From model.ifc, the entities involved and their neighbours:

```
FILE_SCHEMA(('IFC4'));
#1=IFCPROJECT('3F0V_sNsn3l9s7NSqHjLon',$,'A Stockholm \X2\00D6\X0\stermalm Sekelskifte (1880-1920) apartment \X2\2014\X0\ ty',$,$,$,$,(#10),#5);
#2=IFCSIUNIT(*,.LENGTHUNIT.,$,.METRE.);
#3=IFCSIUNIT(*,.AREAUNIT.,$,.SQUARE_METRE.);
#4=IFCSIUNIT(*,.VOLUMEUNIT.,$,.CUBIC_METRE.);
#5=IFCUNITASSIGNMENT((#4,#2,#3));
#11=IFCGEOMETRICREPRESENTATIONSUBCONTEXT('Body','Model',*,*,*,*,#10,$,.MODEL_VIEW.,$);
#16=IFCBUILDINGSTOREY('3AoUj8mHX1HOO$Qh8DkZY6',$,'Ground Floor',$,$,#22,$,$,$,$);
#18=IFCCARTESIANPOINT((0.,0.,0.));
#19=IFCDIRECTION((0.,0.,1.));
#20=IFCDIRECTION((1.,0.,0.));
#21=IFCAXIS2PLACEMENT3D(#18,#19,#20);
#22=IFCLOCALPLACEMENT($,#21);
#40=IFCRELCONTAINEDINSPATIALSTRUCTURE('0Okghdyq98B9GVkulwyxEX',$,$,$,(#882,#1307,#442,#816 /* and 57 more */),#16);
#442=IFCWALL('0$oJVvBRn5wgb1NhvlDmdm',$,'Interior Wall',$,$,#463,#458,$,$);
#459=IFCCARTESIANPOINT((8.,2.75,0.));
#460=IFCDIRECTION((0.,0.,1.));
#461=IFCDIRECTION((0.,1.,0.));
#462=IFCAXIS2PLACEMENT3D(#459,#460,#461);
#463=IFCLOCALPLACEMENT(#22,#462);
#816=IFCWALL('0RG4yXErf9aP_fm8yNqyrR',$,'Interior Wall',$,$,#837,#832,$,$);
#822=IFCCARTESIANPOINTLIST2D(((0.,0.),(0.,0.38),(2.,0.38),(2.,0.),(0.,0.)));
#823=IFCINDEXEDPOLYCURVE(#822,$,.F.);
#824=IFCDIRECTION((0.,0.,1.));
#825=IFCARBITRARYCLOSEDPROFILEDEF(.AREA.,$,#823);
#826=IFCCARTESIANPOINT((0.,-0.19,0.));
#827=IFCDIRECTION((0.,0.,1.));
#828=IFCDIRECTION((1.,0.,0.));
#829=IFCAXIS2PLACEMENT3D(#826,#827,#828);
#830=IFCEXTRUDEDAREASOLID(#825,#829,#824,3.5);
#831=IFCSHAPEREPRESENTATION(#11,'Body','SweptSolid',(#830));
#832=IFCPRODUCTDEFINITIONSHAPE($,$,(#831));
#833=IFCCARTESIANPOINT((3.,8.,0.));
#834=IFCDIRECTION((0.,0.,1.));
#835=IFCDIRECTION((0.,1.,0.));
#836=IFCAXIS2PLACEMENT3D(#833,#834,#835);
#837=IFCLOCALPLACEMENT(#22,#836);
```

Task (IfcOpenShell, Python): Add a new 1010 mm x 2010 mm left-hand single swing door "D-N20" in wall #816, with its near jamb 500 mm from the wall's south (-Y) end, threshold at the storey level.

```python
import numpy as np
import ifcopenshell
import ifcopenshell.api.feature
import ifcopenshell.api.geometry
import ifcopenshell.api.root
import ifcopenshell.api.spatial
import ifcopenshell.geom
import ifcopenshell.util.element
import ifcopenshell.util.placement
import ifcopenshell.util.representation
import ifcopenshell.util.shape
import ifcopenshell.util.unit

model = ifcopenshell.open("model.ifc")
unit_scale = ifcopenshell.util.unit.calculate_unit_scale(model)
settings = ifcopenshell.geom.settings()


def volume(element):
    """Net volume in cubic metres, openings subtracted."""
    shape = ifcopenshell.geom.create_shape(settings, element)
    return ifcopenshell.util.shape.get_volume(shape.geometry)


wall = model.by_guid("0RG4yXErf9aP_fm8yNqyrR")
storey = ifcopenshell.util.element.get_container(wall, ifc_class="IfcBuildingStorey")
context = ifcopenshell.util.representation.get_context(model, "Model", "Body", "MODEL_VIEW")
before = volume(wall)

width, height, from_end, sill = 1.01, 2.01, 0.5, 0.0  # metres

# The wall runs along its own X axis, and the end named is its -X end.
wall_shape = ifcopenshell.geom.create_shape(settings, wall)
x, y, z = ifcopenshell.util.shape.get_vertices(wall_shape.geometry).T
start = x.min() + from_end
face, thickness = float(y.min()), float(y.max() - y.min())
wall_matrix = ifcopenshell.util.placement.get_local_placement(wall.ObjectPlacement)
level = ifcopenshell.util.placement.get_local_placement(storey.ObjectPlacement)[2, 3]


def in_wall(x, y):
    """Placement at x, y metres in the wall's axes, at sill height."""
    matrix = wall_matrix.copy()
    matrix[:, 3] = wall_matrix @ np.array([x / unit_scale, y / unit_scale, 0.0, 1.0])
    matrix[2, 3] = level + sill / unit_scale
    return matrix


# Opening: a box that overshoots both wall faces by 50 mm.
opening = ifcopenshell.api.root.create_entity(model, ifc_class="IfcOpeningElement", predefined_type="OPENING")
box = ifcopenshell.api.geometry.add_wall_representation(
    model, context=context, length=width, height=height, thickness=thickness + 0.1
)
ifcopenshell.api.geometry.assign_representation(model, product=opening, representation=box)
ifcopenshell.api.geometry.edit_object_placement(model, product=opening, matrix=in_wall(start, face - 0.05), is_si=False)
ifcopenshell.api.feature.add_feature(model, feature=opening, element=wall)

door = ifcopenshell.api.root.create_entity(model, ifc_class="IfcDoor", name="D-N20", predefined_type="DOOR")
door.OverallWidth, door.OverallHeight = width / unit_scale, height / unit_scale
door.OperationType = "SINGLE_SWING_LEFT"
body = ifcopenshell.api.geometry.add_door_representation(
    model,
    context=context,
    overall_width=door.OverallWidth,
    overall_height=door.OverallHeight,
    operation_type="SINGLE_SWING_LEFT",
    lining_properties={"LiningDepth": thickness / unit_scale, "ThresholdDepth": thickness / unit_scale},
)
ifcopenshell.api.geometry.assign_representation(model, product=door, representation=body)
ifcopenshell.api.spatial.assign_container(model, products=[door], relating_structure=storey)
ifcopenshell.api.feature.add_filling(model, opening=opening, element=door)

# The lining spans the wall, so the door starts at the wall face.
ifcopenshell.api.geometry.edit_object_placement(model, product=door, matrix=in_wall(start, face), is_si=False)

after = volume(wall)

print(f"wall volume {before:.3f} -> {after:.3f} m3")

model.write("model_updated.ifc")
```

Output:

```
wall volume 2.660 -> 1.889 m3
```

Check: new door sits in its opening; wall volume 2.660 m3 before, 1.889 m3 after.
